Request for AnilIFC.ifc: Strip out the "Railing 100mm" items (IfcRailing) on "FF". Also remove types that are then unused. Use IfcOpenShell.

First a look at what the model holds.

```python
import ifcopenshell
import ifcopenshell.util.element

model = ifcopenshell.open("AnilIFC.ifc")
print(model.schema)
storey = next(s for s in model.by_type("IfcBuildingStorey") if s.Name == "FF")
railings = [e for e in ifcopenshell.util.element.get_decomposition(storey) if e.is_a("IfcRailing")]
seen = {}
for e in railings:
    element_type = ifcopenshell.util.element.get_type(e)
    name = element_type.Name if element_type not in (None, e) else None
    seen[name] = seen.get(name, 0) + 1
for name, count in sorted(seen.items(), key=str):
    print(count, "x", name)
```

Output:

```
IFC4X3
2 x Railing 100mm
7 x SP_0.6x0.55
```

```python
import ifcopenshell
import ifcopenshell.api.root
import ifcopenshell.util.element

model = ifcopenshell.open("AnilIFC.ifc")

storey = next(s for s in model.by_type("IfcBuildingStorey") if s.Name == "FF")
railings = [e for e in ifcopenshell.util.element.get_decomposition(storey) if e.is_a("IfcRailing")]
targets = [e for e in railings if (t := ifcopenshell.util.element.get_type(e)) not in (None, e) and t.Name == "Railing 100mm"]
types = {ifcopenshell.util.element.get_type(e) for e in targets} - {None, *targets}

for e in targets:
    ifcopenshell.api.root.remove_product(model, product=e)
print(len(targets), "removed")

unused = [t for t in types if not ifcopenshell.util.element.get_types(t)]
for t in unused:
    ifcopenshell.api.root.remove_product(model, product=t)
print(len(unused), "unused types removed")

model.write("AnilIFC_v2.ifc")
```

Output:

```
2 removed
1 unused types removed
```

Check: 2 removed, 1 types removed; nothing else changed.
